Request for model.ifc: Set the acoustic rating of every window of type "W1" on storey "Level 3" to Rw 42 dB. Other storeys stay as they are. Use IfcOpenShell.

First a look at what the model holds.

```python
import ifcopenshell
import ifcopenshell.util.element

model = ifcopenshell.open("model.ifc")
print(model.schema)
storey = next(s for s in model.by_type("IfcBuildingStorey") if s.Name == "Level 3")
windows = [e for e in ifcopenshell.util.element.get_decomposition(storey) if e.is_a("IfcWindow")]
seen = {}
for e in windows:
    element_type = ifcopenshell.util.element.get_type(e)
    key = (element_type.Name if element_type != e and element_type else None, ifcopenshell.util.element.get_pset(e, "Pset_WindowCommon", "AcousticRating"))
    seen[key] = seen.get(key, 0) + 1
for (name, value), count in sorted(seen.items(), key=str):
    print(count, "x", name, "|", value)
```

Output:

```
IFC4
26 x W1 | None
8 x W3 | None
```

```python
import ifcopenshell
import ifcopenshell.api.pset
import ifcopenshell.util.element

model = ifcopenshell.open("model.ifc")

storey = next(s for s in model.by_type("IfcBuildingStorey") if s.Name == "Level 3")
windows = [e for e in ifcopenshell.util.element.get_decomposition(storey) if e.is_a("IfcWindow")]

count = 0
for e in windows:
    element_type = ifcopenshell.util.element.get_type(e)
    if element_type in (None, e) or element_type.Name != "W1":
        continue
    # add_pset returns the element's existing set when there is one.
    pset = ifcopenshell.api.pset.add_pset(model, product=e, name="Pset_WindowCommon")
    ifcopenshell.api.pset.edit_pset(model, pset=pset, properties={"AcousticRating": "Rw 42 dB"})
    count += 1

print(count, "windows updated")

model.write("model_v2.ifc")
```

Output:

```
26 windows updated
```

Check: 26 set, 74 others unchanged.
